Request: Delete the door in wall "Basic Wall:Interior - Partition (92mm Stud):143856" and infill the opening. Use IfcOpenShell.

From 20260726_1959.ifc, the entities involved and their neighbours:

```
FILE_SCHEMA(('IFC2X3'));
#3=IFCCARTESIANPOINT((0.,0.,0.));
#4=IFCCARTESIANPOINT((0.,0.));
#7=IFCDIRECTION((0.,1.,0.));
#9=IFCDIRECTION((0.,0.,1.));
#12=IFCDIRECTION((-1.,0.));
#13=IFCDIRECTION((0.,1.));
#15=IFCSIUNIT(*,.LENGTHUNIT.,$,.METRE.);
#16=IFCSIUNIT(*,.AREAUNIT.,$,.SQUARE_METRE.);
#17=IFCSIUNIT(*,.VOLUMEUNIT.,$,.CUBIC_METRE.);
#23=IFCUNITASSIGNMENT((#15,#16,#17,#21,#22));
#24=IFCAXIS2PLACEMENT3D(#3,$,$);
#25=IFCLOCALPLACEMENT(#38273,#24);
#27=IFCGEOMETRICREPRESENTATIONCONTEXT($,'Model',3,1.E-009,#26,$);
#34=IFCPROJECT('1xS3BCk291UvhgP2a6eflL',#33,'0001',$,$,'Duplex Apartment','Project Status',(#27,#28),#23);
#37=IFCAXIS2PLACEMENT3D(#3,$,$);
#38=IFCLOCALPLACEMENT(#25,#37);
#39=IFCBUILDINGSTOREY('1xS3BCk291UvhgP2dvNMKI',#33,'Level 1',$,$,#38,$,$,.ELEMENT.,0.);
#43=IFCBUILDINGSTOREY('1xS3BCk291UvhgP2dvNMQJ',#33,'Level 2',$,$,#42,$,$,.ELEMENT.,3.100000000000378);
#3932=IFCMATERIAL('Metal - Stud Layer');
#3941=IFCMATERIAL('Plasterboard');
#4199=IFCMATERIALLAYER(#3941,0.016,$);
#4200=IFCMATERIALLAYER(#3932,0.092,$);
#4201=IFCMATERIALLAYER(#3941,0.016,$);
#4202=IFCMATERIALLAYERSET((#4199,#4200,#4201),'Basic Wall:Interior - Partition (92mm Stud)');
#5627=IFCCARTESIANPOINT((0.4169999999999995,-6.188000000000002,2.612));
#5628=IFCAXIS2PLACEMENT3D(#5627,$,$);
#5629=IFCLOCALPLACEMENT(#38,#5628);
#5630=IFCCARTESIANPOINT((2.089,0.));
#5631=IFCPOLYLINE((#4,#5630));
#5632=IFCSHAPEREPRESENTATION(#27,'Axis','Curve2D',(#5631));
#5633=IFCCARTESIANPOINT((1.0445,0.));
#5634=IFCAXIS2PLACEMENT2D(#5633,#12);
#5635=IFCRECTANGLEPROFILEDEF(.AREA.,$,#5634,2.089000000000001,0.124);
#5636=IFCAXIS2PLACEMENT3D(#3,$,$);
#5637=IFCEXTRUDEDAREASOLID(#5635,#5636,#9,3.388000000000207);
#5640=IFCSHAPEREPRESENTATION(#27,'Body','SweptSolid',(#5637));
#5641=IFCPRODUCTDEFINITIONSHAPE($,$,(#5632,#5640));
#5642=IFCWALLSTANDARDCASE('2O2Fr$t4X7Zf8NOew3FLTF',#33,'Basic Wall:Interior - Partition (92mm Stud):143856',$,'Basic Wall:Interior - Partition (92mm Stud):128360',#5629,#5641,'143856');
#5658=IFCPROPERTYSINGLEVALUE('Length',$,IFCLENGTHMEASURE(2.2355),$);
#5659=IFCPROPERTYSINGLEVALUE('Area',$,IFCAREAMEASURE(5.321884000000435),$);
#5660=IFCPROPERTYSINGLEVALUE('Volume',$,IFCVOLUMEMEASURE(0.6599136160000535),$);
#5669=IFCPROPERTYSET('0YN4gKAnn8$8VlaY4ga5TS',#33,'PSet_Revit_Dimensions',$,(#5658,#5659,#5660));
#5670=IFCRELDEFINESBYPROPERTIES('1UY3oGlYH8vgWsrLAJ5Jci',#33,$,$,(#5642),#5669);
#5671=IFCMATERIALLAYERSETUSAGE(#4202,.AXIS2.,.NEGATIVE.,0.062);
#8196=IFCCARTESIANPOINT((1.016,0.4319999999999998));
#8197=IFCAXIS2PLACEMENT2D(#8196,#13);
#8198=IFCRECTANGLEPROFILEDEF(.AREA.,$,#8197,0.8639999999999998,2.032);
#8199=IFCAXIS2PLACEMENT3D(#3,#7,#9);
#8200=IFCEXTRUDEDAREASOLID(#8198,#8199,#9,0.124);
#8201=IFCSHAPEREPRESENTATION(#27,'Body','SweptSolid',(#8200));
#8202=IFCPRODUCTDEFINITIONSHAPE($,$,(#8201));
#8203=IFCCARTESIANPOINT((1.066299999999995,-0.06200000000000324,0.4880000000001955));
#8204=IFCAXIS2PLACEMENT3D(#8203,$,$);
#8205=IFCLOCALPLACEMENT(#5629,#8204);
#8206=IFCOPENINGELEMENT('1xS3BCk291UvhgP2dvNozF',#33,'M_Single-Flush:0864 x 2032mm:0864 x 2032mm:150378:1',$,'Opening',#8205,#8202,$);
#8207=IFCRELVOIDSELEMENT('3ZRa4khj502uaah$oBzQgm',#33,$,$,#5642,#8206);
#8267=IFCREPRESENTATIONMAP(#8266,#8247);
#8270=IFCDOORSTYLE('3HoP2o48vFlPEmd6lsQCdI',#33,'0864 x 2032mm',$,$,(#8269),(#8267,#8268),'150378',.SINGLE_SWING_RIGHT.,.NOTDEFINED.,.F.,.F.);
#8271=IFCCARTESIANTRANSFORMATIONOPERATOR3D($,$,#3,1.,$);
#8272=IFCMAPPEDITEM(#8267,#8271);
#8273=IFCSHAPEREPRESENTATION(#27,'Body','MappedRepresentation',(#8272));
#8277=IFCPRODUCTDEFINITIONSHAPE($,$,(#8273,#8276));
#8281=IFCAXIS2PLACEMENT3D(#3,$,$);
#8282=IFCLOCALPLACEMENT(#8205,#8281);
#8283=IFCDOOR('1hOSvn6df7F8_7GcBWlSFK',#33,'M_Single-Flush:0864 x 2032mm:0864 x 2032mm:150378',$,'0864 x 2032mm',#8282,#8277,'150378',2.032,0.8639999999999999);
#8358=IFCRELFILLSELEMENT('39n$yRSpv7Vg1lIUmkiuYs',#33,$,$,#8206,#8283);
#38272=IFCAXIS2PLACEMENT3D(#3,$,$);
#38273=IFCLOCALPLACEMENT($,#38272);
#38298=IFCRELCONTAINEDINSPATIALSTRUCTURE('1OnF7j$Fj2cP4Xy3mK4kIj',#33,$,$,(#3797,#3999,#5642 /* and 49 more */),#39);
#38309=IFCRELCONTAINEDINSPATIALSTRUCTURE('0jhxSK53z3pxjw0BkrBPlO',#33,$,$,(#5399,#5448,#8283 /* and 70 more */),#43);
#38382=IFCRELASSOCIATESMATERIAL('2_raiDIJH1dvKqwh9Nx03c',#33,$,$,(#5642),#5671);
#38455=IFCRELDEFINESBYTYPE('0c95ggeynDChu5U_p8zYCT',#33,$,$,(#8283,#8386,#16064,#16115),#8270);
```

```python
import ifcopenshell
import ifcopenshell.api.feature
import ifcopenshell.api.pset
import ifcopenshell.api.root
import ifcopenshell.geom
import ifcopenshell.util.element
import ifcopenshell.util.shape
import ifcopenshell.util.unit

model = ifcopenshell.open("20260726_1959.ifc")
area_scale = ifcopenshell.util.unit.calculate_unit_scale(model, "AREAUNIT")
volume_scale = ifcopenshell.util.unit.calculate_unit_scale(model, "VOLUMEUNIT")
settings = ifcopenshell.geom.settings()


def volume(element):
    """Net volume in cubic metres, openings subtracted."""
    shape = ifcopenshell.geom.create_shape(settings, element)
    return ifcopenshell.util.shape.get_volume(shape.geometry)


door = model.by_guid("1hOSvn6df7F8_7GcBWlSFK")
opening = door.FillsVoids[0].RelatingOpeningElement
wall = opening.VoidsElements[0].RelatingBuildingElement
before = volume(wall)

ifcopenshell.api.root.remove_product(model, product=door)
ifcopenshell.api.feature.remove_feature(model, feature=opening)

after = volume(wall)
thickness = 0.124  # wall thickness in metres

# Update the wall's stored quantities.
pset = model.by_id(ifcopenshell.util.element.get_pset(wall, "PSet_Revit_Dimensions", should_inherit=False)["id"])
ifcopenshell.api.pset.edit_pset(model, pset=pset, properties={
    "Area": model.create_entity("IfcAreaMeasure", after / thickness / area_scale),
    "Volume": model.create_entity("IfcVolumeMeasure", after / volume_scale),
})

print(f"wall volume {before:.3f} -> {after:.3f} m3")

model.write("20260726_1959_v2.ifc")
```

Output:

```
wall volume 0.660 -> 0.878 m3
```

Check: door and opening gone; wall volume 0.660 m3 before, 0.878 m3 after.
